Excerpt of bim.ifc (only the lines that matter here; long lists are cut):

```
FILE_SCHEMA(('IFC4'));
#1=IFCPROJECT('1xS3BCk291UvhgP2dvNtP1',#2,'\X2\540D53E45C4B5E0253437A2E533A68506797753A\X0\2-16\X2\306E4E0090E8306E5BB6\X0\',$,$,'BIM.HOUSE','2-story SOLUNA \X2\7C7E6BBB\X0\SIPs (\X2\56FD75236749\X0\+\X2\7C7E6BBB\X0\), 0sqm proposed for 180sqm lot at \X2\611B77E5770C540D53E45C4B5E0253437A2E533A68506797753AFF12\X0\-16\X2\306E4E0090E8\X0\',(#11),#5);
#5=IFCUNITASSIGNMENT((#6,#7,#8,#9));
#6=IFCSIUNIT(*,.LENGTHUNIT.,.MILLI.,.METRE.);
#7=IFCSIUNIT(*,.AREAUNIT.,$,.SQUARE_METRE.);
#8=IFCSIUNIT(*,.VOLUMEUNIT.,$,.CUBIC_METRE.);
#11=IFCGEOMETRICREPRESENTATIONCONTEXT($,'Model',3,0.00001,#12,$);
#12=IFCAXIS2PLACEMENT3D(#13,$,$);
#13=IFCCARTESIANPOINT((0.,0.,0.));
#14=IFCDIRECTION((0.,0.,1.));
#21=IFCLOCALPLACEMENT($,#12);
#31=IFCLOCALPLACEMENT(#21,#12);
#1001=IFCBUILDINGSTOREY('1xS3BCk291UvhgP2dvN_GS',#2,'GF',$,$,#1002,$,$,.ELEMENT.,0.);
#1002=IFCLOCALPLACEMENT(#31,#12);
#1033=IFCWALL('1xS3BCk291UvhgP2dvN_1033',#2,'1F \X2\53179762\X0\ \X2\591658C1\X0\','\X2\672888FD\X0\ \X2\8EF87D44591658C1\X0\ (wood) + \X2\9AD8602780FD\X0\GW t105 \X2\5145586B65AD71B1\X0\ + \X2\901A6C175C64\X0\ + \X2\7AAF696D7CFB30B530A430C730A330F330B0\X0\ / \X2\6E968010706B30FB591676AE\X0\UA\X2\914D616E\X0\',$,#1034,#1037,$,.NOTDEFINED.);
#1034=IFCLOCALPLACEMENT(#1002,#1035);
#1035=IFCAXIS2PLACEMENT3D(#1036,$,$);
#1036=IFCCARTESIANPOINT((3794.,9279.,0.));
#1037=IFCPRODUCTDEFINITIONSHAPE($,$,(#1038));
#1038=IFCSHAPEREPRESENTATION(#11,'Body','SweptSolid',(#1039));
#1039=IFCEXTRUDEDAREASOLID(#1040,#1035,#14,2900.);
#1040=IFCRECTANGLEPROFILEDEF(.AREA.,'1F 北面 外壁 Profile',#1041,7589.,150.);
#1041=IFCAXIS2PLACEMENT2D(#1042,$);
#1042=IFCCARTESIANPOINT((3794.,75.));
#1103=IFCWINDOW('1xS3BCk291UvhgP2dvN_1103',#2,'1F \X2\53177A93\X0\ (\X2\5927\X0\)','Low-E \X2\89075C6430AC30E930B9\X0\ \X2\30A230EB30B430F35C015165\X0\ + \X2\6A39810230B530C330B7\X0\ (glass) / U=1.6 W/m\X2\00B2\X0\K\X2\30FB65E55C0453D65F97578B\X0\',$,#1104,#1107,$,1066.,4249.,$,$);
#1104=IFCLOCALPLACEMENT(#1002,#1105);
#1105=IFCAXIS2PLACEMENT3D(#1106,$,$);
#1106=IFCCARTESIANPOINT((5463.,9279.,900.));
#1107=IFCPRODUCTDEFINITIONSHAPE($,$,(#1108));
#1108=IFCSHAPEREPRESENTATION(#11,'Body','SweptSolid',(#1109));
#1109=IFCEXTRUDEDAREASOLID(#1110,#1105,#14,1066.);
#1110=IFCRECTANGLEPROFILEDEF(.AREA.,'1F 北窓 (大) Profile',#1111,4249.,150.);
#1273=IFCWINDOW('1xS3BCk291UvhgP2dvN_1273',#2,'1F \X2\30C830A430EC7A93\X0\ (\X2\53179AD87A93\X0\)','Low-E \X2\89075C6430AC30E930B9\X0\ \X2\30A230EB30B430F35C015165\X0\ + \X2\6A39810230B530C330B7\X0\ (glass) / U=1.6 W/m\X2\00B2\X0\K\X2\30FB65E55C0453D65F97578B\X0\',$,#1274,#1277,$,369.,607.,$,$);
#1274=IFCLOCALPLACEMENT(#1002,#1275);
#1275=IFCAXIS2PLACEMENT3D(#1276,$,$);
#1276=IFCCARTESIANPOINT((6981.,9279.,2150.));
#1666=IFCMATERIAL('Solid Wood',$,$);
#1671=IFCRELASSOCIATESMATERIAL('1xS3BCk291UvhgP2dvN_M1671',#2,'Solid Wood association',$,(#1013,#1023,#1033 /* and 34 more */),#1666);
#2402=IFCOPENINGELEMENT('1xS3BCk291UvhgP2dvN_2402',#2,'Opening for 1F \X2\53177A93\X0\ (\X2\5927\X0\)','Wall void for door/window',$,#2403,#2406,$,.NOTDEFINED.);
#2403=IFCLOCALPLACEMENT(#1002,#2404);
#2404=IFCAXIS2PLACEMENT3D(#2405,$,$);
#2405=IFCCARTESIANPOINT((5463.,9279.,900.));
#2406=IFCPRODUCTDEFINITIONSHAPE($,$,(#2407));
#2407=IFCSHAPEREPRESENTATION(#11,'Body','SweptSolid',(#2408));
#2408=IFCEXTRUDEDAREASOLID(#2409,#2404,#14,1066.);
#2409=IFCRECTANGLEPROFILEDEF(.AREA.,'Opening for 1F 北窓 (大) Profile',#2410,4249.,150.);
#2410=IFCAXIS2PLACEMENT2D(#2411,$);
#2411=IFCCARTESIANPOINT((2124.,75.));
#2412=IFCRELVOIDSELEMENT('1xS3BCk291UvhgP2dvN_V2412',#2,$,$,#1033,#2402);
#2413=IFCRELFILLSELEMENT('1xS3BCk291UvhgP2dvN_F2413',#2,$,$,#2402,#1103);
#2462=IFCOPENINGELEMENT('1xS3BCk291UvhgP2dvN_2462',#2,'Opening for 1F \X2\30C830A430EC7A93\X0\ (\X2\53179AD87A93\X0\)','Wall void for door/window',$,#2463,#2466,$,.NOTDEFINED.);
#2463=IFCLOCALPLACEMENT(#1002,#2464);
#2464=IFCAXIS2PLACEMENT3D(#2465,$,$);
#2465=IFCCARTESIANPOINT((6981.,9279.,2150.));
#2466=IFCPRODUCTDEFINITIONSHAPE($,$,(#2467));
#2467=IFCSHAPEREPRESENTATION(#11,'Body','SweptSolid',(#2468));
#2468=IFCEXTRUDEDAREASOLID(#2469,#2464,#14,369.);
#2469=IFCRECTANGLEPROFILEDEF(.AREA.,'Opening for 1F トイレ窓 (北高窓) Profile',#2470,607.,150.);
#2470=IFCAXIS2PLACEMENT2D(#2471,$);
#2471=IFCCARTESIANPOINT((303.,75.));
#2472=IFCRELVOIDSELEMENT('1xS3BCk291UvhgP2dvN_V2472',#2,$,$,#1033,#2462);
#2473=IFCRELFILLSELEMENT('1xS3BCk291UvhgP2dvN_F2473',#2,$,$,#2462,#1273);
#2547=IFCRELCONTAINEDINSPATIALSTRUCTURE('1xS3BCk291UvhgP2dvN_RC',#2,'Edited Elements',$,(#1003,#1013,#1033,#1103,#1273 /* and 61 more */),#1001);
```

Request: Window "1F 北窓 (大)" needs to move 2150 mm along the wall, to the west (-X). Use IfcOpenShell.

```python
import ifcopenshell
import ifcopenshell.api.geometry
import ifcopenshell.util.placement

model = ifcopenshell.open("bim.ifc")

window = model.by_guid("1xS3BCk291UvhgP2dvN_1103")
opening = window.FillsVoids[0].RelatingOpeningElement
wall = opening.VoidsElements[0].RelatingBuildingElement

wall_matrix = ifcopenshell.util.placement.get_local_placement(wall.ObjectPlacement)
shift = wall_matrix[:3, 0] * -2150.0
before = ifcopenshell.util.placement.get_local_placement(window.ObjectPlacement)[:3, 3].copy()

# The window is not placed relative to its opening, so move both.
for product in (opening, window):
    matrix = ifcopenshell.util.placement.get_local_placement(product.ObjectPlacement)
    matrix[:3, 3] += shift
    ifcopenshell.api.geometry.edit_object_placement(model, product=product, matrix=matrix, is_si=False)

after = ifcopenshell.util.placement.get_local_placement(window.ObjectPlacement)[:3, 3]
print("window moved by", (after - before).round(3) + 0.0)

model.write("bim_edited.ifc")
```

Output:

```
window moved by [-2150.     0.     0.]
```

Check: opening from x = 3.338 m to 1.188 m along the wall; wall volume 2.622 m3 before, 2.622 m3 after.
